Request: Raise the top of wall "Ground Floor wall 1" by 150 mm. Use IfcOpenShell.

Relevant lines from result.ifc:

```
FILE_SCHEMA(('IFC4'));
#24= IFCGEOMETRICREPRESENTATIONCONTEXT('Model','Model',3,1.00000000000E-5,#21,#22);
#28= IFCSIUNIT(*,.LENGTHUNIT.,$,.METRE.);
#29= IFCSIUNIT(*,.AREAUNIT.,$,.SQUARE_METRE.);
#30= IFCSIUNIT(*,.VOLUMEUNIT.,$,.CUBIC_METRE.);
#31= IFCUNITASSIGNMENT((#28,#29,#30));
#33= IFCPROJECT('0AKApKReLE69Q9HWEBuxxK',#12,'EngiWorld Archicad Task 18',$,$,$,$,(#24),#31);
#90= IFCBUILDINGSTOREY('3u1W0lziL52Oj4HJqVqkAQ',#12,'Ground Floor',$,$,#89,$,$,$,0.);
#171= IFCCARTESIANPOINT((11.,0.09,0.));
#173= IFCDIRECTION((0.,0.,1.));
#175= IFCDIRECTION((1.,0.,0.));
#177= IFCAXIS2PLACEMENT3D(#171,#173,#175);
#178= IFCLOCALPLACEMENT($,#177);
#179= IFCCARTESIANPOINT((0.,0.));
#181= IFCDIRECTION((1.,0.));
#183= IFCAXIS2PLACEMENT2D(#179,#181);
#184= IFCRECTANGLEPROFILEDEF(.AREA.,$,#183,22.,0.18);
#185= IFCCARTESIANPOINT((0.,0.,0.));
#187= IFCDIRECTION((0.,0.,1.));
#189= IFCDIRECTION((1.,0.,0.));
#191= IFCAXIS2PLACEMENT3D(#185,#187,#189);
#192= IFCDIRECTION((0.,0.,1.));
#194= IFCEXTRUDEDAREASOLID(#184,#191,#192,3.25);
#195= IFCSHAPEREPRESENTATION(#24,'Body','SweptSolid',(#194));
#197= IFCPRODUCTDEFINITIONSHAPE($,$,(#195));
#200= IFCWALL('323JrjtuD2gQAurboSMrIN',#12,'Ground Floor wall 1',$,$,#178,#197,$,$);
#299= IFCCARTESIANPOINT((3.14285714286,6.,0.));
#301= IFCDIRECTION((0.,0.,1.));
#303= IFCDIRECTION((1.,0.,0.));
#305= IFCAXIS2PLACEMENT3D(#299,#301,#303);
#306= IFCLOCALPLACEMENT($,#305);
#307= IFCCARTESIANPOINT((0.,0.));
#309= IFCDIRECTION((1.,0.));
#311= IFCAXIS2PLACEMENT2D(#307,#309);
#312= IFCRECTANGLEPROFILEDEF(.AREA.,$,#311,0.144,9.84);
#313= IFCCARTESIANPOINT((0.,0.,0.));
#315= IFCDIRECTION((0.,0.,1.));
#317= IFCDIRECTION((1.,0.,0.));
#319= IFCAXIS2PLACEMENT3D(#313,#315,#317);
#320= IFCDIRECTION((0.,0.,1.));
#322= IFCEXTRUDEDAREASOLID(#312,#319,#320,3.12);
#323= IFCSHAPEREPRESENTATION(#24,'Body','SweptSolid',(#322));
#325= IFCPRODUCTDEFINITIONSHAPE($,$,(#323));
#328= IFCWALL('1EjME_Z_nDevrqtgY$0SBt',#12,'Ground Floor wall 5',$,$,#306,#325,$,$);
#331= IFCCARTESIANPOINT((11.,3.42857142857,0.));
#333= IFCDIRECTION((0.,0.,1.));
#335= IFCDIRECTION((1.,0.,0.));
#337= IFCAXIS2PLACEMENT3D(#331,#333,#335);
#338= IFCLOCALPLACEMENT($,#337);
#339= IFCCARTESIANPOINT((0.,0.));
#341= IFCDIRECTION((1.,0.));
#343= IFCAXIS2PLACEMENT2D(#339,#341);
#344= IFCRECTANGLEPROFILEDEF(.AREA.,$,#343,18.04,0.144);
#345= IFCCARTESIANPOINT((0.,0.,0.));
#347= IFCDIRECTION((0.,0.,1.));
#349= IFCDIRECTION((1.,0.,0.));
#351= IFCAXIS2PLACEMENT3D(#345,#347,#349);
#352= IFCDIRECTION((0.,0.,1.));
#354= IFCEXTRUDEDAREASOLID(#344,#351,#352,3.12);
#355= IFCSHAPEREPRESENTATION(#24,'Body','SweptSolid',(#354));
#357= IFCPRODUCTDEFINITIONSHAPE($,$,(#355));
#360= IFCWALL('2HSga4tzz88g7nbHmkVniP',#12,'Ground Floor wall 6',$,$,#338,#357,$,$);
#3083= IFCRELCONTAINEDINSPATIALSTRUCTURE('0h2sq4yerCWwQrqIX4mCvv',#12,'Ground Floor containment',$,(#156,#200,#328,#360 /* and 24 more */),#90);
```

```python
import ifcopenshell
import ifcopenshell.geom
import ifcopenshell.util.shape
import ifcopenshell.util.unit

model = ifcopenshell.open("result.ifc")
unit_scale = ifcopenshell.util.unit.calculate_unit_scale(model)
settings = ifcopenshell.geom.settings()


def volume(element):
    """Net volume in cubic metres, openings subtracted."""
    shape = ifcopenshell.geom.create_shape(settings, element)
    return ifcopenshell.util.shape.get_volume(shape.geometry)


wall = model.by_id(200)
before = volume(wall)

body = next(r for r in wall.Representation.Representations if r.RepresentationIdentifier == "Body")
solid = body.Items[0]
old_height = solid.Depth
solid.Depth += 0.15 / unit_scale
after = volume(wall)

print(f"height {old_height:g} -> {solid.Depth:g}, volume {before:.3f} -> {after:.3f} m3")

model.write("result-out.ifc")
```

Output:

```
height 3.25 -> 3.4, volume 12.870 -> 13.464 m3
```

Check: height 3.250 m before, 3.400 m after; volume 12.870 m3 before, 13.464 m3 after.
